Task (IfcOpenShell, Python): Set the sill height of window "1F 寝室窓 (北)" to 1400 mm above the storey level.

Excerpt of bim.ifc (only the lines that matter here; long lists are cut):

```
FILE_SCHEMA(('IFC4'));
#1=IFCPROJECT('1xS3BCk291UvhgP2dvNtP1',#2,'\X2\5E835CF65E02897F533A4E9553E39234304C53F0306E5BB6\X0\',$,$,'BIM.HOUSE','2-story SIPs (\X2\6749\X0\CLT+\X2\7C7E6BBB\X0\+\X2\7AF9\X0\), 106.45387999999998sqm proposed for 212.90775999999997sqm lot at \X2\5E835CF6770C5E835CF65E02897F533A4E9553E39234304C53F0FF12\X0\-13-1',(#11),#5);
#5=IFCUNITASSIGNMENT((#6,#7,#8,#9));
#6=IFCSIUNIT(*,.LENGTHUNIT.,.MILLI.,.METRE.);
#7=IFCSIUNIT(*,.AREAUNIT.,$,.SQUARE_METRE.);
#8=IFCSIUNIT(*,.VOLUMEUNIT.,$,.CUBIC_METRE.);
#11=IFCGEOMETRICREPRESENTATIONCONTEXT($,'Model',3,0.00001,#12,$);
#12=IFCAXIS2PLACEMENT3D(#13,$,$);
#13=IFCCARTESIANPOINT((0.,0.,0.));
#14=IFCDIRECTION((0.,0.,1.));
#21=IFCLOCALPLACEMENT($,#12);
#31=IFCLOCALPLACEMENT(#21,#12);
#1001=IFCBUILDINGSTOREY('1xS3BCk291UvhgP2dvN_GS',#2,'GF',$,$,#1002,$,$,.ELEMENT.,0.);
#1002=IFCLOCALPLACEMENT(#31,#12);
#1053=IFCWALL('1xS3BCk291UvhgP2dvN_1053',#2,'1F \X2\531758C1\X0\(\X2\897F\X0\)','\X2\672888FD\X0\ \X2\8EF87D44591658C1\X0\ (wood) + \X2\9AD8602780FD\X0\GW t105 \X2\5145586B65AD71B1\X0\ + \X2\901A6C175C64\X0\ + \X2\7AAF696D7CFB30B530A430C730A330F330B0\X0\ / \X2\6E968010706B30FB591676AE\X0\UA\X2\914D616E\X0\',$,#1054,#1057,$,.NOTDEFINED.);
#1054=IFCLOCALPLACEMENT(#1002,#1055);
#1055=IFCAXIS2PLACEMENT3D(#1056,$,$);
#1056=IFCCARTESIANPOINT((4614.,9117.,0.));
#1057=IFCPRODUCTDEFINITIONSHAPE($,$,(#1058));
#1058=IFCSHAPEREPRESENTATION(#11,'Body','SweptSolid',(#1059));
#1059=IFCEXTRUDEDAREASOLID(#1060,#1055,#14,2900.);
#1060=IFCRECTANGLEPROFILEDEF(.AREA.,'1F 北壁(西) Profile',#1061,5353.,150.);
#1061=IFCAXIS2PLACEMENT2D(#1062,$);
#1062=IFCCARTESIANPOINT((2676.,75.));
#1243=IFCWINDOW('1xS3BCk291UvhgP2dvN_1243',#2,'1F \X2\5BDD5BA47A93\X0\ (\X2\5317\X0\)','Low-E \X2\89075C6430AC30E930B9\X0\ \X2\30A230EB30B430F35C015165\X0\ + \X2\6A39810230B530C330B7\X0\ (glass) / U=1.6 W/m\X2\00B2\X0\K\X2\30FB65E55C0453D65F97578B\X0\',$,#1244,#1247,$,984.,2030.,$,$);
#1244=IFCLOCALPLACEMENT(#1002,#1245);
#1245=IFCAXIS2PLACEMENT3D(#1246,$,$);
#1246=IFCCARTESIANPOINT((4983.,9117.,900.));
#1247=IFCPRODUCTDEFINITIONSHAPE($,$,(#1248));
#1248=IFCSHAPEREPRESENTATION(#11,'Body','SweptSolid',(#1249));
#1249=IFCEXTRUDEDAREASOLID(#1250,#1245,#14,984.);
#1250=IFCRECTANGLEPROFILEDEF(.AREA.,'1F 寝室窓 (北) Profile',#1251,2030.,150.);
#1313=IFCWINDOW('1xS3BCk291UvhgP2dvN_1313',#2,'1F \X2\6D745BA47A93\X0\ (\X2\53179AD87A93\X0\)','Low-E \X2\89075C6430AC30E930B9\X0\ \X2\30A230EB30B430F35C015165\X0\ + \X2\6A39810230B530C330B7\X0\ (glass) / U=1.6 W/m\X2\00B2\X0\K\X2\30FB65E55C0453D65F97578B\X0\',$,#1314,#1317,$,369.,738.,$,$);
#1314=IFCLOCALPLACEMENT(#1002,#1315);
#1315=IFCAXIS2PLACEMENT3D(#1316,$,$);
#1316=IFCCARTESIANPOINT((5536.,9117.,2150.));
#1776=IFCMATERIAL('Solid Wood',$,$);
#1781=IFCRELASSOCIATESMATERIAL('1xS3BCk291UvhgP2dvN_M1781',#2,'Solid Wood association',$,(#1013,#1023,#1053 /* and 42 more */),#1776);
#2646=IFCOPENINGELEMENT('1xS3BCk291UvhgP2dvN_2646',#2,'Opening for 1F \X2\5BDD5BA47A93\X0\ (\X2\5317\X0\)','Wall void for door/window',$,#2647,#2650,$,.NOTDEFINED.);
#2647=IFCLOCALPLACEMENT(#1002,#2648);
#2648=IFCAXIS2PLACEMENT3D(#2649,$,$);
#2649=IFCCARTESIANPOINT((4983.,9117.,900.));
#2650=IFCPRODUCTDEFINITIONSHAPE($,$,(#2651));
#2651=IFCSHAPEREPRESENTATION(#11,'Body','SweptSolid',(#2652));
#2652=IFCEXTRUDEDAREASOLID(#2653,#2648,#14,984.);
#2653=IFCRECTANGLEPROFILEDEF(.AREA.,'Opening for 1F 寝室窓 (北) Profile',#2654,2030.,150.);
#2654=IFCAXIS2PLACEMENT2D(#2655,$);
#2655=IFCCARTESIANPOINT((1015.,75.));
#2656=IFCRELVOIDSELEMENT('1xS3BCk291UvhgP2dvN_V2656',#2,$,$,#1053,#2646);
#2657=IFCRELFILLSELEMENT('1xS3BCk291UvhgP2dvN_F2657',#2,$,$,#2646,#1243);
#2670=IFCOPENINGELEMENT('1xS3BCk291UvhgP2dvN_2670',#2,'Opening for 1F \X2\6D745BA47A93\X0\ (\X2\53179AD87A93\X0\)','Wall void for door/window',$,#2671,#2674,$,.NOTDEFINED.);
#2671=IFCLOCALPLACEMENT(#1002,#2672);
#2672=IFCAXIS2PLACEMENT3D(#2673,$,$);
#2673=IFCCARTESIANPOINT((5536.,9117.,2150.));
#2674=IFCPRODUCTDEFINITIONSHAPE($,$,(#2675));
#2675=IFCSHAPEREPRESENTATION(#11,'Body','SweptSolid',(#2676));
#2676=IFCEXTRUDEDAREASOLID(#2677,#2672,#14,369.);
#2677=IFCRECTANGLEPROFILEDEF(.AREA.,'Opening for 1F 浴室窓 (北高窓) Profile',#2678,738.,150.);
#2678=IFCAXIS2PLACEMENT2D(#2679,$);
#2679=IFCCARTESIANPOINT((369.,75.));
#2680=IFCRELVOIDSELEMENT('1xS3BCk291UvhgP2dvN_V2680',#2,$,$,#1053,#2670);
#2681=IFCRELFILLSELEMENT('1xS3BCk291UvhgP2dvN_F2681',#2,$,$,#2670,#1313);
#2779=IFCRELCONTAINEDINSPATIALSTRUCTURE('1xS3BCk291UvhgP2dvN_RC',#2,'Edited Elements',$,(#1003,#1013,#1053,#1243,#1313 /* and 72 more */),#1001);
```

```python
import numpy as np
import ifcopenshell
import ifcopenshell.api.geometry
import ifcopenshell.geom
import ifcopenshell.util.element
import ifcopenshell.util.placement
import ifcopenshell.util.shape
import ifcopenshell.util.unit

model = ifcopenshell.open("bim.ifc")
unit_scale = ifcopenshell.util.unit.calculate_unit_scale(model)

window = model.by_id(1243)
opening = window.FillsVoids[0].RelatingOpeningElement
storey = ifcopenshell.util.element.get_container(window, ifc_class="IfcBuildingStorey")
level = ifcopenshell.util.placement.get_local_placement(storey.ObjectPlacement)[2, 3]

# The opening's origin need not be at the sill, so measure its lowest point.
shape = ifcopenshell.geom.create_shape(ifcopenshell.geom.settings(), opening)
bottom = ifcopenshell.util.shape.get_shape_bottom_elevation(shape, shape.geometry) / unit_scale
dz = level + 1.4 / unit_scale - bottom

shift = np.array([0.0, 0.0, dz])
# The window is not placed relative to its opening, so move both.
for product in (opening, window):
    matrix = ifcopenshell.util.placement.get_local_placement(product.ObjectPlacement)
    matrix[:3, 3] += shift
    ifcopenshell.api.geometry.edit_object_placement(model, product=product, matrix=matrix, is_si=False)

print(f"moved by {dz * unit_scale:+.3f} m")

model.write("bim_rev.ifc")
```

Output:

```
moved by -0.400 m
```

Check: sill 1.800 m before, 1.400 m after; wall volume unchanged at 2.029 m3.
